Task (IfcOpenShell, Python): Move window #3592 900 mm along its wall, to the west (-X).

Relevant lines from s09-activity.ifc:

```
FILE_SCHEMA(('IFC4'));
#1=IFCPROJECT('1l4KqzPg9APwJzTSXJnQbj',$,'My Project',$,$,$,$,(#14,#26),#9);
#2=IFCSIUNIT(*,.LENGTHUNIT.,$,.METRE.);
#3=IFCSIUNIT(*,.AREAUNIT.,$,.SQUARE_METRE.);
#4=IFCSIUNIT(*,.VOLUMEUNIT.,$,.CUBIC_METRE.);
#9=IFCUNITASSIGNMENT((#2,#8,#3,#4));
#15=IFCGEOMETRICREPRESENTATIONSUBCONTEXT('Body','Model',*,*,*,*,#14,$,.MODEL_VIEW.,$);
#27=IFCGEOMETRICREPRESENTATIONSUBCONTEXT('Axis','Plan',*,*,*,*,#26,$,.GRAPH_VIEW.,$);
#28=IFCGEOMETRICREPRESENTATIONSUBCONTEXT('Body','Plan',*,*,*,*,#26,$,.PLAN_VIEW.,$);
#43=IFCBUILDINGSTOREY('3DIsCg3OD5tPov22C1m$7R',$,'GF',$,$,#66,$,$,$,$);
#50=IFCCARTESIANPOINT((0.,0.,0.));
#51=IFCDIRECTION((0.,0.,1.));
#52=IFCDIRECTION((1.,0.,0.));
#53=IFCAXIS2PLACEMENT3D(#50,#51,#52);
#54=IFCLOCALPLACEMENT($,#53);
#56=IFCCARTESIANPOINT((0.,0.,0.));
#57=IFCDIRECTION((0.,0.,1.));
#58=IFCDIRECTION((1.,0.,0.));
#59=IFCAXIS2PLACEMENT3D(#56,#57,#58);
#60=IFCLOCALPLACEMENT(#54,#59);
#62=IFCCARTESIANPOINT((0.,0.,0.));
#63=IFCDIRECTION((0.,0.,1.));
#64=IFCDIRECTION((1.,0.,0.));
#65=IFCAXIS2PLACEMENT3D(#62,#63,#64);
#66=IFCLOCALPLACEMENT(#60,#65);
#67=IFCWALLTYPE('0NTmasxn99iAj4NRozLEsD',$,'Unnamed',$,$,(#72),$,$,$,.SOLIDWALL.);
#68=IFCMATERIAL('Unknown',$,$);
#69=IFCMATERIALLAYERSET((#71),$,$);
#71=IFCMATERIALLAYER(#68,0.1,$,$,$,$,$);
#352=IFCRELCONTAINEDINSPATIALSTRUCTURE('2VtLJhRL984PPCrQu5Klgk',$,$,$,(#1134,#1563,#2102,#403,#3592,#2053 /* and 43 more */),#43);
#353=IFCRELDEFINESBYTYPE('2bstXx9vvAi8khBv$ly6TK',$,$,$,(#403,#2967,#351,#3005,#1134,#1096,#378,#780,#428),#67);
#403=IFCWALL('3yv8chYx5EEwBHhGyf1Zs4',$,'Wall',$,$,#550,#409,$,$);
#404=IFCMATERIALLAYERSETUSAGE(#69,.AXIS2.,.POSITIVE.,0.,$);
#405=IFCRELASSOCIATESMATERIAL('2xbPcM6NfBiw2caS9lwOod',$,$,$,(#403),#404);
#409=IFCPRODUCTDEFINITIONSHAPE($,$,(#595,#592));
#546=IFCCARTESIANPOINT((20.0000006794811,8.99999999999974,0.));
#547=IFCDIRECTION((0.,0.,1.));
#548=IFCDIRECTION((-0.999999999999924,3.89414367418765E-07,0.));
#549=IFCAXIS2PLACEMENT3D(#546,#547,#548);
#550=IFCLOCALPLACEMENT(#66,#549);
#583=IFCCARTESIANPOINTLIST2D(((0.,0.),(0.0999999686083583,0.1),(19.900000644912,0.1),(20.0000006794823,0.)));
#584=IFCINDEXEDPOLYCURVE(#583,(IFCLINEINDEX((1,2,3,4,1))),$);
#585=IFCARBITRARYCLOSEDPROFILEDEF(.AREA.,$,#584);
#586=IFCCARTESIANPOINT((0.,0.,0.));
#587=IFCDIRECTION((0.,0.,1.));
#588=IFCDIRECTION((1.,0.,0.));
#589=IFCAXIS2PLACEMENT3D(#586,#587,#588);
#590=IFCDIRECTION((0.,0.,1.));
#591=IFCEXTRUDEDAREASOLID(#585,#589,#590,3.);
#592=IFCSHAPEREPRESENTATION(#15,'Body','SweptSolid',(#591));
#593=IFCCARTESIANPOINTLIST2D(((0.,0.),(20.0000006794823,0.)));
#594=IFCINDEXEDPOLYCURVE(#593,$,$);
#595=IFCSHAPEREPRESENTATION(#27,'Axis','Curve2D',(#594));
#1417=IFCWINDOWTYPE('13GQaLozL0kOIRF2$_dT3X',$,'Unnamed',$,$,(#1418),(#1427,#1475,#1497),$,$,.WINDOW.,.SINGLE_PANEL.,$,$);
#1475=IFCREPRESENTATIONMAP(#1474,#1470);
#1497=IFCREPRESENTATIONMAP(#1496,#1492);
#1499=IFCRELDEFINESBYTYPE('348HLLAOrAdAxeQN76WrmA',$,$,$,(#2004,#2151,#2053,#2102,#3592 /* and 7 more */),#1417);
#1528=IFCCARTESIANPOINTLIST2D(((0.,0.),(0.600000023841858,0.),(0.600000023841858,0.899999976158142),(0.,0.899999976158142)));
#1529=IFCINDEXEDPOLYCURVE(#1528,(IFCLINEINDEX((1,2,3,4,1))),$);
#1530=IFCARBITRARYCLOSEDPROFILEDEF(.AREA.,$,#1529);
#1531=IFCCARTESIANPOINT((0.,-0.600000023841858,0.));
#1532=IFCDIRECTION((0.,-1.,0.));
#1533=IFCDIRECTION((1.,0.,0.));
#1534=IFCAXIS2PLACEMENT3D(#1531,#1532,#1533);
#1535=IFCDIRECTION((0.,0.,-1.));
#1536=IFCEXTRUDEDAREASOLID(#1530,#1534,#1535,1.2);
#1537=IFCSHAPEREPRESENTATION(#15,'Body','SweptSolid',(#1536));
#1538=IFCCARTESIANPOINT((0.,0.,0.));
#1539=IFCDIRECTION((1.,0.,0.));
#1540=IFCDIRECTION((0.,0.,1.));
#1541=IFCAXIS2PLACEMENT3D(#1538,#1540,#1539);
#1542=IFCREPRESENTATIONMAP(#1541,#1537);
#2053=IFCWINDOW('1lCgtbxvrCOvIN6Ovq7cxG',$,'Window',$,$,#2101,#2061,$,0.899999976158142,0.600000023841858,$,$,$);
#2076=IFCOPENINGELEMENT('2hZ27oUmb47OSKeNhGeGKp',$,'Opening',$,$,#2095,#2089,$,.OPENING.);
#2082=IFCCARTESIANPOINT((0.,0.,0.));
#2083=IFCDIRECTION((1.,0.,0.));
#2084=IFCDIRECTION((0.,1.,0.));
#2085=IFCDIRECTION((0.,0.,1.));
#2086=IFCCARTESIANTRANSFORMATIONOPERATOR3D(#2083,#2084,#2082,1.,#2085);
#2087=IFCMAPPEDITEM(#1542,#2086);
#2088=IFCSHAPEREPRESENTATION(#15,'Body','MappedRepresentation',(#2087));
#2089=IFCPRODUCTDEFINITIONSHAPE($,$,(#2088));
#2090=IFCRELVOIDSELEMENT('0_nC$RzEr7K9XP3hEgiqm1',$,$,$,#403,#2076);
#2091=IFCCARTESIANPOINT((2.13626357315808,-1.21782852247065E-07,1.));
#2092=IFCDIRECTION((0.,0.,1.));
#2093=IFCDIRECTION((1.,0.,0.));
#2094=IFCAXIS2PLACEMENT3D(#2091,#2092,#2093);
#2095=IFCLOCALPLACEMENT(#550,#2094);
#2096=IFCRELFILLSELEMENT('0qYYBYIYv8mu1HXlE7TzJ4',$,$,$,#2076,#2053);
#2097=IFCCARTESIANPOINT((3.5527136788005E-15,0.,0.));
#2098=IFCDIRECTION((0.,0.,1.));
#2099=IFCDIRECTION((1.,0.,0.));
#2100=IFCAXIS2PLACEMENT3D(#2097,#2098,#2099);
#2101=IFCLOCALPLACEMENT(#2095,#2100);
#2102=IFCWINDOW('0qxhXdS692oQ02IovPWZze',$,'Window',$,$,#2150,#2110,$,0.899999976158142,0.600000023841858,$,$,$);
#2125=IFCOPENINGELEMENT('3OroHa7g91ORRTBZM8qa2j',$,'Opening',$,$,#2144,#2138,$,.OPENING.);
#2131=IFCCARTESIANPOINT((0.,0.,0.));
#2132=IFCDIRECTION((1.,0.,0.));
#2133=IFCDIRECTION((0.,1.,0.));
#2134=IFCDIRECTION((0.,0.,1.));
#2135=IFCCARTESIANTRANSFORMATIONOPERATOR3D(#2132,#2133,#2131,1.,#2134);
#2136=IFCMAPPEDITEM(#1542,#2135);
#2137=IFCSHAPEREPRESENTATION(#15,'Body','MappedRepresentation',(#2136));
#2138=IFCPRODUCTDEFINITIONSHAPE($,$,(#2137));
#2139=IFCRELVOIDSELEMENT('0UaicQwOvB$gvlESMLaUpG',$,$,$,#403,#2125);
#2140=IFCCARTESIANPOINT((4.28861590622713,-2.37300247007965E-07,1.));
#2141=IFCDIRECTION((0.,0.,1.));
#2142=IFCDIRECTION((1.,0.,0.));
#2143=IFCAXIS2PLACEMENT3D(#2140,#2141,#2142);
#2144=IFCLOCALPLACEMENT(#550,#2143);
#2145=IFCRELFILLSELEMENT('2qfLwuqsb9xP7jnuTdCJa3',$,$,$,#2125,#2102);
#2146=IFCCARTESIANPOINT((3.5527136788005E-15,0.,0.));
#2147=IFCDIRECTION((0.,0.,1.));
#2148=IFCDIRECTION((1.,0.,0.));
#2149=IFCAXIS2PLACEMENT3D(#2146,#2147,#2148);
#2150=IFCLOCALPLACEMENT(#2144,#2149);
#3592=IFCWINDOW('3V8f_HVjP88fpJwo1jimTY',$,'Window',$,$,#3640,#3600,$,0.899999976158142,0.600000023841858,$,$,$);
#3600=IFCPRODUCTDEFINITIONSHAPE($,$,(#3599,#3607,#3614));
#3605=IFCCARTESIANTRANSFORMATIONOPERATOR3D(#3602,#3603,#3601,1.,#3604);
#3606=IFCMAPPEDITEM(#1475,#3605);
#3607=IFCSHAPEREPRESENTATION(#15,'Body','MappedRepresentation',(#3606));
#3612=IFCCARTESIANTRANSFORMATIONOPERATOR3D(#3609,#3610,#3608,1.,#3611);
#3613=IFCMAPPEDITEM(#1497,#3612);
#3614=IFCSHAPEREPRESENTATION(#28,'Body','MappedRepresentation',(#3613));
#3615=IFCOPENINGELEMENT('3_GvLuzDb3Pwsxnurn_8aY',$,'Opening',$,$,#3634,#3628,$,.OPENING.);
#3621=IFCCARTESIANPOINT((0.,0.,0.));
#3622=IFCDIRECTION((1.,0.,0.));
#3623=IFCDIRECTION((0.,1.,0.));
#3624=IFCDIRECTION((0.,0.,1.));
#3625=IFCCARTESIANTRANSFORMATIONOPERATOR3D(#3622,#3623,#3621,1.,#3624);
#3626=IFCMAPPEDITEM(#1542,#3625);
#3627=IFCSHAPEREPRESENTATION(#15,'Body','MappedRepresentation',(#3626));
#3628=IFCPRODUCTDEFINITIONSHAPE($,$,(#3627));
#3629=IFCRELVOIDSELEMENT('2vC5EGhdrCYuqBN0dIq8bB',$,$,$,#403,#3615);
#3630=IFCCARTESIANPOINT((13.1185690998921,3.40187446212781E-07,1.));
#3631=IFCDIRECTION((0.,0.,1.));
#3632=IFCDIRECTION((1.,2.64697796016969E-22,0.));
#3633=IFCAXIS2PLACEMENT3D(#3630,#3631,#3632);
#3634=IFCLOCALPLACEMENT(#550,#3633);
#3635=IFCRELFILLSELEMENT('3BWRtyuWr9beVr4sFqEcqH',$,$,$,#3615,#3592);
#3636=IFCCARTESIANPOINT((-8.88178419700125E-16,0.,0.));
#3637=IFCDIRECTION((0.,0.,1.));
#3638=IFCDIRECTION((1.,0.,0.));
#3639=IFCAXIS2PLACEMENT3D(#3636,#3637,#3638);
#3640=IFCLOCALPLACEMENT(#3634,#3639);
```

```python
import ifcopenshell
import ifcopenshell.api.geometry
import ifcopenshell.util.placement
import ifcopenshell.util.unit

model = ifcopenshell.open("s09-activity.ifc")
unit_scale = ifcopenshell.util.unit.calculate_unit_scale(model)

window = model.by_guid("3V8f_HVjP88fpJwo1jimTY")
opening = window.FillsVoids[0].RelatingOpeningElement
wall = opening.VoidsElements[0].RelatingBuildingElement

wall_matrix = ifcopenshell.util.placement.get_local_placement(wall.ObjectPlacement)
shift = wall_matrix[:3, 0] * 0.9 / unit_scale
before = ifcopenshell.util.placement.get_local_placement(window.ObjectPlacement)[:3, 3].copy()

# The window is placed relative to its opening, so it follows when the opening moves.
matrix = ifcopenshell.util.placement.get_local_placement(opening.ObjectPlacement)
matrix[:3, 3] += shift
ifcopenshell.api.geometry.edit_object_placement(
    model, product=opening, matrix=matrix, is_si=False, should_transform_children=True
)

after = ifcopenshell.util.placement.get_local_placement(window.ObjectPlacement)[:3, 3]
print("window moved by", (after - before).round(3) + 0.0)

model.write("s09-activity_v2.ifc")
```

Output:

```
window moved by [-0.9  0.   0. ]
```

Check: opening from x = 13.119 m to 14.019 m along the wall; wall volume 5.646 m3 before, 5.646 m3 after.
